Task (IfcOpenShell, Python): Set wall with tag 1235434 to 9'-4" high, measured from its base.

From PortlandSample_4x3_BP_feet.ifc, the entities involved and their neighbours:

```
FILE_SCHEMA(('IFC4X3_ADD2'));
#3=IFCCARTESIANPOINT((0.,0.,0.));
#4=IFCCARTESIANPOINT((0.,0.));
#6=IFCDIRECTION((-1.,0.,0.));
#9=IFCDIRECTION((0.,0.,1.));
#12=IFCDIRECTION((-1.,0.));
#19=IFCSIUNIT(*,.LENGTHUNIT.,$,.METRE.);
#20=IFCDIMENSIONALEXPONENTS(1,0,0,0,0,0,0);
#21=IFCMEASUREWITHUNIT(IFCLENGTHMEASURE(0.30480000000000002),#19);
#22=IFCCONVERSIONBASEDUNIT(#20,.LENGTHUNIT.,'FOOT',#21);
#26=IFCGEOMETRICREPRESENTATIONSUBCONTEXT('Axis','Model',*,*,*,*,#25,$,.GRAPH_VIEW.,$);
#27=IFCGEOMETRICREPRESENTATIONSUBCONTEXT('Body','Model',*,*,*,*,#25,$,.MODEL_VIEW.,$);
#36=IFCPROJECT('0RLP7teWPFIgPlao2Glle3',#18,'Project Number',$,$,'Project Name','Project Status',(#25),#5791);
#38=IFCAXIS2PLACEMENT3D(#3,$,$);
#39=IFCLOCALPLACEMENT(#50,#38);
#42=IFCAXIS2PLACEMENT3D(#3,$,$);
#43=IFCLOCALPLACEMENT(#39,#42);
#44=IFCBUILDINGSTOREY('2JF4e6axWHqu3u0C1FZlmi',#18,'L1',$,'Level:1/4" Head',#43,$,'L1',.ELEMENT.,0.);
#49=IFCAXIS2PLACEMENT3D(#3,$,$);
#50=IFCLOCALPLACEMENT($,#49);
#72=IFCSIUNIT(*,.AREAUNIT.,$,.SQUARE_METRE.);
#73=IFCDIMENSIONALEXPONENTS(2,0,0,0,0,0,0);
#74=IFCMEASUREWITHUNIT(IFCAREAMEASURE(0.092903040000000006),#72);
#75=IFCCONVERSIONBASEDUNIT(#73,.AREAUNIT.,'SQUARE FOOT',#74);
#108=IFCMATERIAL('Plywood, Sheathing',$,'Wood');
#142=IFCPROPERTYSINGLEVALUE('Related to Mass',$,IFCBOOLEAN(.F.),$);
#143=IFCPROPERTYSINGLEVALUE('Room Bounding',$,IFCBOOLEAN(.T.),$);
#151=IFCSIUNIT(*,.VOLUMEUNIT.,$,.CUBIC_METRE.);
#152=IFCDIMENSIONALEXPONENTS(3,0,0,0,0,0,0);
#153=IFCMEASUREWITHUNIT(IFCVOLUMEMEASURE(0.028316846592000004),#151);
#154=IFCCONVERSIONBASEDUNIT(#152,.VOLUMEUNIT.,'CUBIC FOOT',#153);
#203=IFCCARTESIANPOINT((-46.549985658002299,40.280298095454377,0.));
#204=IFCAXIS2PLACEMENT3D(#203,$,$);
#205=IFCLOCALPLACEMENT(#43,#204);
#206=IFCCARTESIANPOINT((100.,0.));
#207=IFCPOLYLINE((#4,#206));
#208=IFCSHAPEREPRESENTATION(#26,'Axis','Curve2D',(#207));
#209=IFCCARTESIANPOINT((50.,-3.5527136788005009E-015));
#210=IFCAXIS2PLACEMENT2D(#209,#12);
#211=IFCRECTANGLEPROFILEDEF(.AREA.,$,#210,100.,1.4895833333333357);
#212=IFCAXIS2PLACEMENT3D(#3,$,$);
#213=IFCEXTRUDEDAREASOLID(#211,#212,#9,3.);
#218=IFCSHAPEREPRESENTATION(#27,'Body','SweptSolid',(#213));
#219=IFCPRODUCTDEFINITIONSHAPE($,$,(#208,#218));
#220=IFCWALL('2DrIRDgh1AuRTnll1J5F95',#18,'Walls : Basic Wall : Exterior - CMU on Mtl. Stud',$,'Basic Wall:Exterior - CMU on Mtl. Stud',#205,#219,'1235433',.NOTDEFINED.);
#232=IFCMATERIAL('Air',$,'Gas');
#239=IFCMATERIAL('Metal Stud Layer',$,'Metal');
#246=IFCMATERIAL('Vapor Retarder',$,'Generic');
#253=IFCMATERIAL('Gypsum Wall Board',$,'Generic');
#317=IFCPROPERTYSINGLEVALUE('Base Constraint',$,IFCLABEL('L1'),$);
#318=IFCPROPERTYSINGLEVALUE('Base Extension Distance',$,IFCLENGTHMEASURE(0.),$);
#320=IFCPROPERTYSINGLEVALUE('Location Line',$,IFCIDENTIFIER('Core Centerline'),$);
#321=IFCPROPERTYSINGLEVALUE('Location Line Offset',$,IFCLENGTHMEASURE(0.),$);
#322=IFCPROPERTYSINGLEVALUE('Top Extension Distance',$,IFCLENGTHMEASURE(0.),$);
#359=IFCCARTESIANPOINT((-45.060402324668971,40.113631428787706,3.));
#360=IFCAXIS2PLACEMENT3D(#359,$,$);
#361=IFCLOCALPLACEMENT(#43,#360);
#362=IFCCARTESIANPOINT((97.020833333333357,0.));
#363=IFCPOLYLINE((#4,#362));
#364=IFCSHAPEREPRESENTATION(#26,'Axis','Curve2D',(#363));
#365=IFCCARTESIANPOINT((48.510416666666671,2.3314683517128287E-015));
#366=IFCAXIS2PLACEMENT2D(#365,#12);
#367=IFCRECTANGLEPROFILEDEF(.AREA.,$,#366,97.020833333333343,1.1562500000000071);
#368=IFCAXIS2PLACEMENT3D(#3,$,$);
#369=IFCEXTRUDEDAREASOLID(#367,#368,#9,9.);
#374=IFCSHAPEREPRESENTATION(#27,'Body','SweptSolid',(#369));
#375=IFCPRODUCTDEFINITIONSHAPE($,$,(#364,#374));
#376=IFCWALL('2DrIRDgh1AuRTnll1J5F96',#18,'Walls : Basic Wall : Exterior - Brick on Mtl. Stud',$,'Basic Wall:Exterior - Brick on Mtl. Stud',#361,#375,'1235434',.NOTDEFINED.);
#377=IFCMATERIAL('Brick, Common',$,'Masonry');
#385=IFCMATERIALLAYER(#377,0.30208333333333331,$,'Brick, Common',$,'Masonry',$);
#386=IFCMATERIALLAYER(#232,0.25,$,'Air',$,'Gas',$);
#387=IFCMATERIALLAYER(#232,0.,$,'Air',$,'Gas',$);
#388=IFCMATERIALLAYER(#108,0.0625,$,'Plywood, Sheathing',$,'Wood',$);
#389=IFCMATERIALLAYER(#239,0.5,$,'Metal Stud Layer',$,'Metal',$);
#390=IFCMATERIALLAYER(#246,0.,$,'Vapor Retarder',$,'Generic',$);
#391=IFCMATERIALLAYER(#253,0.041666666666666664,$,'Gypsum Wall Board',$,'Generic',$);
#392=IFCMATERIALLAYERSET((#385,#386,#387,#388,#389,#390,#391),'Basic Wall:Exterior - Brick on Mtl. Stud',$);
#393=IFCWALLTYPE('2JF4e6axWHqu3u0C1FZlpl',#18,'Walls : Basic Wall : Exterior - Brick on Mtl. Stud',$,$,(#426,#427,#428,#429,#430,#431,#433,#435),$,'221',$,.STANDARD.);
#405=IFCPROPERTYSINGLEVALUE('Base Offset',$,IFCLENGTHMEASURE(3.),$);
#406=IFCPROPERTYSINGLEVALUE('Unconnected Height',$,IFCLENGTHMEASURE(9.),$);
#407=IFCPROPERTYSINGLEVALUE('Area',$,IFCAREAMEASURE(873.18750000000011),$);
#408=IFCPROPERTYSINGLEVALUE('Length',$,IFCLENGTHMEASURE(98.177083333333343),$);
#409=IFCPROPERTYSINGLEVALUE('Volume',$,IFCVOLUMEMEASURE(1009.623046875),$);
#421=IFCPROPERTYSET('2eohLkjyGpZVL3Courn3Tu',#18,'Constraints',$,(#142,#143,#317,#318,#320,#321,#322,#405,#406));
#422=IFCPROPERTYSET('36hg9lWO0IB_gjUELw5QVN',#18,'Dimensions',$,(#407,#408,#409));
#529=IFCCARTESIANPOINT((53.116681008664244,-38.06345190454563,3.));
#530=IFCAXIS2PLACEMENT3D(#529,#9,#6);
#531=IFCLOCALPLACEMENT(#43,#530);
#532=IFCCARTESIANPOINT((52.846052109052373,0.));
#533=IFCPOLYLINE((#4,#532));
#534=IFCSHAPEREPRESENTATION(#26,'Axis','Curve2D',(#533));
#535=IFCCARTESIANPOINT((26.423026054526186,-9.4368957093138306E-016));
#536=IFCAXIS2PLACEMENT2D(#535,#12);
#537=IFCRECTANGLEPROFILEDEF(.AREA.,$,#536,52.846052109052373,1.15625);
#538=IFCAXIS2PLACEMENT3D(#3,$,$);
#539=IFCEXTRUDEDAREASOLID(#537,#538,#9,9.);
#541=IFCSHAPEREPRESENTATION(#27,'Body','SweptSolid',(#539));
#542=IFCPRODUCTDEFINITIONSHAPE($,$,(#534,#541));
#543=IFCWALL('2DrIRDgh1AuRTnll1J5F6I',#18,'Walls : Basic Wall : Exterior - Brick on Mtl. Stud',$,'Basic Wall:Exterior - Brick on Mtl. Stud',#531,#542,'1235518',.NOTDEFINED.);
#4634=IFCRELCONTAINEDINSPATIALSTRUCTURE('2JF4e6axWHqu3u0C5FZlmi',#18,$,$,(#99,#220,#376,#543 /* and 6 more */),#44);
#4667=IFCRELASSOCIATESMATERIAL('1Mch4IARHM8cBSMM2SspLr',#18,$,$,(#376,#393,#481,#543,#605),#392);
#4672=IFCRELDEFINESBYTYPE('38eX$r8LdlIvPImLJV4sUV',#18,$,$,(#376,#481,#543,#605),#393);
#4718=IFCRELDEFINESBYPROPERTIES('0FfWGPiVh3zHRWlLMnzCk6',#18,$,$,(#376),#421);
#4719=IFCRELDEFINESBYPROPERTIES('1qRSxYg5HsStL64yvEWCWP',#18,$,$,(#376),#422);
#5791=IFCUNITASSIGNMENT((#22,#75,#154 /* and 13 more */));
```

```python
import ifcopenshell
import ifcopenshell.api.pset
import ifcopenshell.geom
import ifcopenshell.util.element
import ifcopenshell.util.representation
import ifcopenshell.util.shape
import ifcopenshell.util.unit

model = ifcopenshell.open("PortlandSample_4x3_BP_feet.ifc")
unit_scale = ifcopenshell.util.unit.calculate_unit_scale(model)
area_scale = ifcopenshell.util.unit.calculate_unit_scale(model, "AREAUNIT")
volume_scale = ifcopenshell.util.unit.calculate_unit_scale(model, "VOLUMEUNIT")
settings = ifcopenshell.geom.settings()


def volume(element):
    """Net volume in cubic metres, openings subtracted."""
    shape = ifcopenshell.geom.create_shape(settings, element)
    return ifcopenshell.util.shape.get_volume(shape.geometry)


wall = model.by_guid("2DrIRDgh1AuRTnll1J5F96")
before = volume(wall)

body = ifcopenshell.util.representation.get_representation(wall, "Model", "Body")
solid = body.Items[0]
old_height = solid.Depth
solid.Depth = 112 * 0.0254 / unit_scale
after = volume(wall)
thickness = 0.3524  # wall thickness in metres

# Update the stored height, areas and volumes.
pset = model.by_id(ifcopenshell.util.element.get_pset(wall, "Constraints", should_inherit=False)["id"])
ifcopenshell.api.pset.edit_pset(model, pset=pset, properties={
    "Unconnected Height": model.create_entity("IfcLengthMeasure", solid.Depth),
})
pset = model.by_id(ifcopenshell.util.element.get_pset(wall, "Dimensions", should_inherit=False)["id"])
ifcopenshell.api.pset.edit_pset(model, pset=pset, properties={
    "Area": model.create_entity("IfcAreaMeasure", after / thickness / area_scale),
    "Volume": model.create_entity("IfcVolumeMeasure", after / volume_scale),
})

print(f"height {old_height:g} -> {solid.Depth:g}, volume {before:.3f} -> {after:.3f} m3")

model.write("PortlandSample_4x3_BP_feet_v2.ifc")
```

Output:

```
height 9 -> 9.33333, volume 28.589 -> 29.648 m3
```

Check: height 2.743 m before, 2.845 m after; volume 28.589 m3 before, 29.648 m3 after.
